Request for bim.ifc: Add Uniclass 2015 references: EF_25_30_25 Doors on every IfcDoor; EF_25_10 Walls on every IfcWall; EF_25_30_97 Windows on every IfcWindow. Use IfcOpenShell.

First a look at what the model holds.

```python
import ifcopenshell

model = ifcopenshell.open("bim.ifc")
print(model.schema)
print("classifications:", [c.Name for c in model.by_type("IfcClassification")])
for ifc_class in ("IfcDoor", "IfcRoof", "IfcStair", "IfcWall", "IfcWindow"):
    print(ifc_class, len(model.by_type(ifc_class)))
```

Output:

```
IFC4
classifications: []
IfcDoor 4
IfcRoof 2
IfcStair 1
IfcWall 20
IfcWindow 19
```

```python
import ifcopenshell
import ifcopenshell.api.classification

model = ifcopenshell.open("bim.ifc")

system = ifcopenshell.api.classification.add_classification(model, classification="Uniclass 2015")

codes = {
    "IfcDoor": ("EF_25_30_25", "Doors"),
    "IfcWall": ("EF_25_10", "Walls"),
    "IfcWindow": ("EF_25_30_97", "Windows"),
}
for ifc_class, (code, name) in codes.items():
    products = model.by_type(ifc_class)
    ifcopenshell.api.classification.add_reference(
        model, products=products, classification=system, identification=code, name=name
    )
    print(code, len(products))

model.write("bim_updated.ifc")
```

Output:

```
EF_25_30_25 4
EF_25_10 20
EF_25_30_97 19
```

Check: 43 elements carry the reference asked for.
